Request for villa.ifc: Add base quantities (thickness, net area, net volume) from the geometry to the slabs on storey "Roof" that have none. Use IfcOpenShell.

First a look at what the model holds.

```python
import ifcopenshell
import ifcopenshell.util.element
import ifcopenshell.util.unit

model = ifcopenshell.open("villa.ifc")
print(model.schema)
for unit_type in ("LENGTHUNIT", "AREAUNIT", "VOLUMEUNIT"):
    print(unit_type, ifcopenshell.util.unit.calculate_unit_scale(model, unit_type))
storey = next(s for s in model.by_type("IfcBuildingStorey") if s.Name == "Roof")
slabs = [e for e in ifcopenshell.util.element.get_decomposition(storey) if e.is_a("IfcSlab")]
for e in sorted(slabs, key=lambda e: e.id()):
    print(e.id(), e.is_a(), e.Name, list(ifcopenshell.util.element.get_psets(e, qtos_only=True)), sep=" | ")
```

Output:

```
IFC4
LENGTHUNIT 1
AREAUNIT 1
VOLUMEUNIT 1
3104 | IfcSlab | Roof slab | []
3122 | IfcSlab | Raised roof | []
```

```python
import ifcopenshell
import ifcopenshell.api.pset
import ifcopenshell.geom
import ifcopenshell.util.element
import ifcopenshell.util.shape
import ifcopenshell.util.unit

model = ifcopenshell.open("villa.ifc")
unit_scale = ifcopenshell.util.unit.calculate_unit_scale(model)
area_scale = ifcopenshell.util.unit.calculate_unit_scale(model, "AREAUNIT")
volume_scale = ifcopenshell.util.unit.calculate_unit_scale(model, "VOLUMEUNIT")
settings = ifcopenshell.geom.settings()

storey = next(s for s in model.by_type("IfcBuildingStorey") if s.Name == "Roof")
slabs = [e for e in ifcopenshell.util.element.get_decomposition(storey) if e.is_a("IfcSlab")]

for e in sorted(slabs, key=lambda e: e.id()):
    if ifcopenshell.util.element.get_psets(e, qtos_only=True, should_inherit=False):
        continue
    # Geometry comes back in metres, in the element's own axes.
    shape = ifcopenshell.geom.create_shape(settings, e)
    values = {
        "Width": ifcopenshell.util.shape.get_z(shape.geometry) / unit_scale,
        "NetArea": ifcopenshell.util.shape.get_footprint_area(shape.geometry) / area_scale,
        "NetVolume": ifcopenshell.util.shape.get_volume(shape.geometry) / volume_scale,
    }
    qto = ifcopenshell.api.pset.add_qto(model, product=e, name="Qto_SlabBaseQuantities")
    ifcopenshell.api.pset.edit_qto(model, qto=qto, properties=values)
    print(e.id(), {k: round(v, 3) for k, v in values.items()})

model.write("villa_updated.ifc")
```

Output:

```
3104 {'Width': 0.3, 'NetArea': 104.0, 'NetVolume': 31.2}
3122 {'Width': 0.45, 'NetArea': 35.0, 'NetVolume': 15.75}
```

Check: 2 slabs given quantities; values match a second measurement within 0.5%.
